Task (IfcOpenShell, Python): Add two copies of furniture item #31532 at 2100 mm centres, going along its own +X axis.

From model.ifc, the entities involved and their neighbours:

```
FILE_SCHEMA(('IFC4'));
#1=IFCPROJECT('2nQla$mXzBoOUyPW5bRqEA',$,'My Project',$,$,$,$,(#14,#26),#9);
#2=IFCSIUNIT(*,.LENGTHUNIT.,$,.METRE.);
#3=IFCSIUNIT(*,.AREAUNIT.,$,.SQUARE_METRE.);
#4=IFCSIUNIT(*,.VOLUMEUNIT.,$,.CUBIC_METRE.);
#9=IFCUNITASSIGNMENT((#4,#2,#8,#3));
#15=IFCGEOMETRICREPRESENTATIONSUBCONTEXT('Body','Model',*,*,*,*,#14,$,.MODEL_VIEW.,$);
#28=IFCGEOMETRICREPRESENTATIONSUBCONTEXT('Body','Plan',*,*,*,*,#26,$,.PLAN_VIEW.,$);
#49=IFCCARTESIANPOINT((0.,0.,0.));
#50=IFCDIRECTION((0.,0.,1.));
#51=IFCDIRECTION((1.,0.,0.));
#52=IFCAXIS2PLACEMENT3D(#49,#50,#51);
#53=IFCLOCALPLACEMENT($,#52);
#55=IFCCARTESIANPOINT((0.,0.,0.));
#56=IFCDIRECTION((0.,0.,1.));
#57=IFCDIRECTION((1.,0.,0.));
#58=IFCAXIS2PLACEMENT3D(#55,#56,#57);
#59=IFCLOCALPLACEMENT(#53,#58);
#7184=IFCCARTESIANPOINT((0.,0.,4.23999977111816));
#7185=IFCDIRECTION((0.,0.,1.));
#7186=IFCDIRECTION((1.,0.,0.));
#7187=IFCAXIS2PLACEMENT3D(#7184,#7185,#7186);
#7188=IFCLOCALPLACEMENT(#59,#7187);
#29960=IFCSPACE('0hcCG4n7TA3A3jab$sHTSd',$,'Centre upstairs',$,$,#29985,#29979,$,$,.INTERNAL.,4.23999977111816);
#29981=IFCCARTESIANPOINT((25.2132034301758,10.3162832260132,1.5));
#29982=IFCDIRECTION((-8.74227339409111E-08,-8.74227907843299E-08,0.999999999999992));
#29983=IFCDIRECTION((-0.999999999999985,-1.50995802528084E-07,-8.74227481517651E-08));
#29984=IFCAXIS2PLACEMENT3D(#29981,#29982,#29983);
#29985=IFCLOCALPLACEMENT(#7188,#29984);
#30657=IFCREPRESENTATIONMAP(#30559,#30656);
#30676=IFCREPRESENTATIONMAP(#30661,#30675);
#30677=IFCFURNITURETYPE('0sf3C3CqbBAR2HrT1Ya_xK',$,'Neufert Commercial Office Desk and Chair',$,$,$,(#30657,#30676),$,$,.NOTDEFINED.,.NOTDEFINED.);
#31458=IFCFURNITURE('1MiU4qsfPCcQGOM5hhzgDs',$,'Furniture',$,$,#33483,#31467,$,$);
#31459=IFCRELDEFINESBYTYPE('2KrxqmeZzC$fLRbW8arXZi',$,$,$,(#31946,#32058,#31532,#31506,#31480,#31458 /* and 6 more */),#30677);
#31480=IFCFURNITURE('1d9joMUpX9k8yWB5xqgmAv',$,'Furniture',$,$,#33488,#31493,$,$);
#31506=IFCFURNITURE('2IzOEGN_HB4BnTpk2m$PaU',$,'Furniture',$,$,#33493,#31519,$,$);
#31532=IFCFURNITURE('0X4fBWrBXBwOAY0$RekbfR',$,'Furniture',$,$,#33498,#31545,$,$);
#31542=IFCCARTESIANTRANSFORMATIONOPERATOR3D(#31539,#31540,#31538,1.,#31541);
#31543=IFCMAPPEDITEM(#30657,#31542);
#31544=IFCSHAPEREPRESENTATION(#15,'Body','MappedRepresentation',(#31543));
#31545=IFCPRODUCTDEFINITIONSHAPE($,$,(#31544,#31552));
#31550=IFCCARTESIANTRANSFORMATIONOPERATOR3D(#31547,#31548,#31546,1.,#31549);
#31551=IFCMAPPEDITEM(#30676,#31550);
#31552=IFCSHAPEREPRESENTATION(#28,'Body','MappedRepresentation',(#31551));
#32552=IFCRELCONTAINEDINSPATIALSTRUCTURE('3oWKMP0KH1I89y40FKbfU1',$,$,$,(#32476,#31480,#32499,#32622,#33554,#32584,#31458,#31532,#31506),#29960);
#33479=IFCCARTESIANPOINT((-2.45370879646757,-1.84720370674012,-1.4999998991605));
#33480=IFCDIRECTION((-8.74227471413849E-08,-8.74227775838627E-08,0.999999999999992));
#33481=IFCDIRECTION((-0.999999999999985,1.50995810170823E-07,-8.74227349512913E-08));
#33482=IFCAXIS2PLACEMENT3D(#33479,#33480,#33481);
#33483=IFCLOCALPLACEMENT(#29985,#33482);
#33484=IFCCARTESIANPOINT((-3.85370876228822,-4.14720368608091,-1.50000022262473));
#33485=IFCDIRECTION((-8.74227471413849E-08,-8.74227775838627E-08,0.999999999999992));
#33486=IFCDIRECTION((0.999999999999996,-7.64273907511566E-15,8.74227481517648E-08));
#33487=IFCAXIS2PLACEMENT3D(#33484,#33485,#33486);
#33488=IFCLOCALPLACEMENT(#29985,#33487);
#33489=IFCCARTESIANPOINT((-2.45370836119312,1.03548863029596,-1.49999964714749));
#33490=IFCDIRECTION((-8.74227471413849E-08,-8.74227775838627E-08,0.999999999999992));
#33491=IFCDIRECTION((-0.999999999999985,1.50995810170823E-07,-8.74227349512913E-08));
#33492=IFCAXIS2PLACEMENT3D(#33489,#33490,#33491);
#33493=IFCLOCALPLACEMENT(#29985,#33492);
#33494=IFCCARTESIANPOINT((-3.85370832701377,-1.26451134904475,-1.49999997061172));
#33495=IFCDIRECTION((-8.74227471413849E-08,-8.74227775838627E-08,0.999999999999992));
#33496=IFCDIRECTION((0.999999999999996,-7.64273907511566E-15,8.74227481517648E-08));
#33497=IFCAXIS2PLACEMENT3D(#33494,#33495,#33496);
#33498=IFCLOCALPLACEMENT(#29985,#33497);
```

```python
import ifcopenshell
import ifcopenshell.api.geometry
import ifcopenshell.api.root
import ifcopenshell.util.element
import ifcopenshell.util.placement

model = ifcopenshell.open("model.ifc")

source = model.by_guid("0X4fBWrBXBwOAY0$RekbfR")
base = ifcopenshell.util.placement.get_local_placement(source.ObjectPlacement)
step = base[:3, 0] * 2.1

for i in range(1, 3):
    copy = ifcopenshell.api.root.copy_class(model, product=source)
    copy.Representation = ifcopenshell.util.element.copy_deep(
        model, source.Representation, exclude=["IfcGeometricRepresentationContext", "IfcRepresentationMap"]
    )
    matrix = base.copy()
    matrix[:3, 3] += i * step
    print("added at", matrix[:3, 3].round(3) + 0.0)
    ifcopenshell.api.geometry.edit_object_placement(model, product=copy, matrix=matrix, is_si=False)

model.write("model-out.ifc")
```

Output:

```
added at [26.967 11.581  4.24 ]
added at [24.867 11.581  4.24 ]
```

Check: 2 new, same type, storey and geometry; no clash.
